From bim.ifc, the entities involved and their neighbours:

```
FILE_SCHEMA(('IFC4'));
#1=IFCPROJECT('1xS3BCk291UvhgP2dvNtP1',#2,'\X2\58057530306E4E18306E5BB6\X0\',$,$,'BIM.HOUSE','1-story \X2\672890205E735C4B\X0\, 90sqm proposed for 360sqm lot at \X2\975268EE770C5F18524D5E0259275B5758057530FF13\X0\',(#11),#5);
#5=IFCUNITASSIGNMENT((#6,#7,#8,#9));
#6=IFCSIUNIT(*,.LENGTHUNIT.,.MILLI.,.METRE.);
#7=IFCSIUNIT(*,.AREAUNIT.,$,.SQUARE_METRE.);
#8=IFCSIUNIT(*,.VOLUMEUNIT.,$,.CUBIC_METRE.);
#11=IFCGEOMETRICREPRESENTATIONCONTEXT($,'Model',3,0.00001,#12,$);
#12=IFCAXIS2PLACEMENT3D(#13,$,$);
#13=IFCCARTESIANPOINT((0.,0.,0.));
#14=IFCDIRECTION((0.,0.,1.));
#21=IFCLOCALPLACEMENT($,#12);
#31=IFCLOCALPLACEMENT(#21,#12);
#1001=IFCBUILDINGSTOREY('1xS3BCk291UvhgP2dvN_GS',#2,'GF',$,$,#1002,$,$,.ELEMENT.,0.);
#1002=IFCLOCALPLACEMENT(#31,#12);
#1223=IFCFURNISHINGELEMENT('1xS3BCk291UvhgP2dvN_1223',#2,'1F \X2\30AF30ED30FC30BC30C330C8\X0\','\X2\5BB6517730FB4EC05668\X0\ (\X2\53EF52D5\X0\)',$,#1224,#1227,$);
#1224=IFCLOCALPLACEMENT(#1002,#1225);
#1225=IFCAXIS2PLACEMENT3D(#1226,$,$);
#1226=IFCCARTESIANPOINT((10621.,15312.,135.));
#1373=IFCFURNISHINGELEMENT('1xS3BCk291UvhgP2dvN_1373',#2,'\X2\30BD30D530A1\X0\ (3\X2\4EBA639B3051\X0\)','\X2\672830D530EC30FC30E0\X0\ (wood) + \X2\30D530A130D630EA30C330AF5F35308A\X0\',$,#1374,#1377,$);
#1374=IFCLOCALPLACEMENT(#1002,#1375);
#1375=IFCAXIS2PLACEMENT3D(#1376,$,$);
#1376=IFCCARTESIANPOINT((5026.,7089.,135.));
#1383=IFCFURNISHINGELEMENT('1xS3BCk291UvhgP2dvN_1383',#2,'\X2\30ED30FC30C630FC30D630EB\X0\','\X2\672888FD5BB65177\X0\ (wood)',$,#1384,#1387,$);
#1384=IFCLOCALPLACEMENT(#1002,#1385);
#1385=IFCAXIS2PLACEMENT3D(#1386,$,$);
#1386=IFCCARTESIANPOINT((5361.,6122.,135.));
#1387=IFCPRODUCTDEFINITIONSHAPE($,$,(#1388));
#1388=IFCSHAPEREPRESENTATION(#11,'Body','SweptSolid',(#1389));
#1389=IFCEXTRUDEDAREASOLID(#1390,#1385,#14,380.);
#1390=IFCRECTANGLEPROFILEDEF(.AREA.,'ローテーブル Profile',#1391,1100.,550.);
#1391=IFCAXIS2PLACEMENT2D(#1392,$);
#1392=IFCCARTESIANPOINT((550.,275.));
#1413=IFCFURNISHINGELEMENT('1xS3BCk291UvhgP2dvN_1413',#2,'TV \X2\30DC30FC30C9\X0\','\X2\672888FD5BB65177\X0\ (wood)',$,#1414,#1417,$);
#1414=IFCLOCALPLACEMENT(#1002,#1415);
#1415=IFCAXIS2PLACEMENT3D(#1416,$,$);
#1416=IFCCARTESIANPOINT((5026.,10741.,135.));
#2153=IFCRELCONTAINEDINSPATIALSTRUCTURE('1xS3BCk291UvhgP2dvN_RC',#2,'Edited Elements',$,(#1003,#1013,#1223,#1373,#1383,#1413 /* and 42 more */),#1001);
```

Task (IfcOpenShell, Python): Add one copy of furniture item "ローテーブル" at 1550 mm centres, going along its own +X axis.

```python
import ifcopenshell
import ifcopenshell.api.geometry
import ifcopenshell.api.root
import ifcopenshell.util.element
import ifcopenshell.util.placement
import ifcopenshell.util.unit

model = ifcopenshell.open("bim.ifc")
unit_scale = ifcopenshell.util.unit.calculate_unit_scale(model)


def reuse_history(source, copy):
    """copy_class also copies each property set's owner history, people and application; keep the originals."""
    for rel in copy.IsDefinedBy:
        if rel.is_a("IfcRelDefinesByProperties") and (history := rel.RelatingPropertyDefinition.OwnerHistory):
            rel.RelatingPropertyDefinition.OwnerHistory = source.OwnerHistory
            ifcopenshell.util.element.remove_deep2(model, history)


source = model.by_id(1383)
base = ifcopenshell.util.placement.get_local_placement(source.ObjectPlacement)
step = base[:3, 0] * 1.55 / unit_scale

for i in range(1, 2):
    copy = ifcopenshell.api.root.copy_class(model, product=source)
    copy.Representation = ifcopenshell.util.element.copy_deep(
        model, source.Representation, exclude=["IfcGeometricRepresentationContext", "IfcRepresentationMap"]
    )
    reuse_history(source, copy)
    matrix = base.copy()
    matrix[:3, 3] += i * step
    print("added at", matrix[:3, 3].round(3) + 0.0)
    ifcopenshell.api.geometry.edit_object_placement(model, product=copy, matrix=matrix, is_si=False)

model.write("bim_edited.ifc")
```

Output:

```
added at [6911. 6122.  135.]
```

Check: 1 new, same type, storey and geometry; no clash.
